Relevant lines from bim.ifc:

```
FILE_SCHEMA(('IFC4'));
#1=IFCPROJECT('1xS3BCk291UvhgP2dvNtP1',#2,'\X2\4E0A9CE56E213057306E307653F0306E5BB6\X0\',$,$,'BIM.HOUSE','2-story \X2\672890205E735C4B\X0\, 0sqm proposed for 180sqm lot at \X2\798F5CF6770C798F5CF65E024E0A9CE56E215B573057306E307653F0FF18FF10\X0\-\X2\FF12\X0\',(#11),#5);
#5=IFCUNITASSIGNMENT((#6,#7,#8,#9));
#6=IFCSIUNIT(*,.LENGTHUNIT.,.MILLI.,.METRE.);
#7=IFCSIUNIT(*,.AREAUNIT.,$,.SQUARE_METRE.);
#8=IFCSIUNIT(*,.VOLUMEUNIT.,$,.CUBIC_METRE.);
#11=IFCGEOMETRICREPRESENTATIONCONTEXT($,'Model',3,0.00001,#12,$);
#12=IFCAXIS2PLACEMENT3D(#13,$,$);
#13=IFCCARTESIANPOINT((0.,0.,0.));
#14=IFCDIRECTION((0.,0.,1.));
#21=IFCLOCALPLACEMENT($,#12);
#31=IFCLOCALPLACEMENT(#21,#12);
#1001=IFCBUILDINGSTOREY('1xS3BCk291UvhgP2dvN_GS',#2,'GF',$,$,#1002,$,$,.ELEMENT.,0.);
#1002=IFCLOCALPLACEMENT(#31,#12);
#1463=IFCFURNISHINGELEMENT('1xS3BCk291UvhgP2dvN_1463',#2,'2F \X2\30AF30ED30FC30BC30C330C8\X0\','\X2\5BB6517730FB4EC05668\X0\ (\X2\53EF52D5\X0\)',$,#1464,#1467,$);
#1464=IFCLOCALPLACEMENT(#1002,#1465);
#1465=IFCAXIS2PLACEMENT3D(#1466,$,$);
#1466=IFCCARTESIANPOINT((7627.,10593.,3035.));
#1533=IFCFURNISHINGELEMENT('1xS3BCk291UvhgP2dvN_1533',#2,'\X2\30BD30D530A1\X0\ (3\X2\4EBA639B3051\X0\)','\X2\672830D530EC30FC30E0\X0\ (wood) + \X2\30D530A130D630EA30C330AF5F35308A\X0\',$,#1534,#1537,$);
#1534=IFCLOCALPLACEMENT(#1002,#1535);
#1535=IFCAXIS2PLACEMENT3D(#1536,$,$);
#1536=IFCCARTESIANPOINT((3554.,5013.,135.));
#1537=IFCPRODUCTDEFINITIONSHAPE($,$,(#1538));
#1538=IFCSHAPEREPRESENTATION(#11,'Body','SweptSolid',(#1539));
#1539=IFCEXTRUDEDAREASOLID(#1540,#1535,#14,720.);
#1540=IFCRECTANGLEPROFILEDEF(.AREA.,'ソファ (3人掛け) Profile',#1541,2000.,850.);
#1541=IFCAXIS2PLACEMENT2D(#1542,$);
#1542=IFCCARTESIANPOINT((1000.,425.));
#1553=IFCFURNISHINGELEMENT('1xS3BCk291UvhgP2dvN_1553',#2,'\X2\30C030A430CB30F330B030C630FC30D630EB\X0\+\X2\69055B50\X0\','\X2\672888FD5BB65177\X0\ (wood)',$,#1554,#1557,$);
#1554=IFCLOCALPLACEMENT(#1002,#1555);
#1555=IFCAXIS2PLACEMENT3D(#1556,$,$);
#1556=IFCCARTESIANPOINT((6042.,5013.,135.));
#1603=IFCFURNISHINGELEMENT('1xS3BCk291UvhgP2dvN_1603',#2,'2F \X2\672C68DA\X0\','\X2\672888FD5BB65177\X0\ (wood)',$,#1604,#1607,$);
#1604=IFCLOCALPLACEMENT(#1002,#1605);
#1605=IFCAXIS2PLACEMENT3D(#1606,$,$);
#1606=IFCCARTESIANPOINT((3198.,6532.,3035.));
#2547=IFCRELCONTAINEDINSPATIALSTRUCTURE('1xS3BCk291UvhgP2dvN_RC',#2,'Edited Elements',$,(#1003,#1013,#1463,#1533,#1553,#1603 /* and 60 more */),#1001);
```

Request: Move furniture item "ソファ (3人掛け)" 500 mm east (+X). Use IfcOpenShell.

```python
import ifcopenshell
import ifcopenshell.api.geometry
import ifcopenshell.util.placement

model = ifcopenshell.open("bim.ifc")

item = model.by_guid("1xS3BCk291UvhgP2dvN_1533")
matrix = ifcopenshell.util.placement.get_local_placement(item.ObjectPlacement)
matrix[0, 3] += 500.0
ifcopenshell.api.geometry.edit_object_placement(model, product=item, matrix=matrix, is_si=False)

print(ifcopenshell.util.placement.get_local_placement(item.ObjectPlacement).round(3) + 0.0)

model.write("bim_v2.ifc")
```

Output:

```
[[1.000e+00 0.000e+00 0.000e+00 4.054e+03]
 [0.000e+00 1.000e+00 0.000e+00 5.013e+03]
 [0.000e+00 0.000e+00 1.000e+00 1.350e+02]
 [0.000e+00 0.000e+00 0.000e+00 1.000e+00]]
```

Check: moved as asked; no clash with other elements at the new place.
